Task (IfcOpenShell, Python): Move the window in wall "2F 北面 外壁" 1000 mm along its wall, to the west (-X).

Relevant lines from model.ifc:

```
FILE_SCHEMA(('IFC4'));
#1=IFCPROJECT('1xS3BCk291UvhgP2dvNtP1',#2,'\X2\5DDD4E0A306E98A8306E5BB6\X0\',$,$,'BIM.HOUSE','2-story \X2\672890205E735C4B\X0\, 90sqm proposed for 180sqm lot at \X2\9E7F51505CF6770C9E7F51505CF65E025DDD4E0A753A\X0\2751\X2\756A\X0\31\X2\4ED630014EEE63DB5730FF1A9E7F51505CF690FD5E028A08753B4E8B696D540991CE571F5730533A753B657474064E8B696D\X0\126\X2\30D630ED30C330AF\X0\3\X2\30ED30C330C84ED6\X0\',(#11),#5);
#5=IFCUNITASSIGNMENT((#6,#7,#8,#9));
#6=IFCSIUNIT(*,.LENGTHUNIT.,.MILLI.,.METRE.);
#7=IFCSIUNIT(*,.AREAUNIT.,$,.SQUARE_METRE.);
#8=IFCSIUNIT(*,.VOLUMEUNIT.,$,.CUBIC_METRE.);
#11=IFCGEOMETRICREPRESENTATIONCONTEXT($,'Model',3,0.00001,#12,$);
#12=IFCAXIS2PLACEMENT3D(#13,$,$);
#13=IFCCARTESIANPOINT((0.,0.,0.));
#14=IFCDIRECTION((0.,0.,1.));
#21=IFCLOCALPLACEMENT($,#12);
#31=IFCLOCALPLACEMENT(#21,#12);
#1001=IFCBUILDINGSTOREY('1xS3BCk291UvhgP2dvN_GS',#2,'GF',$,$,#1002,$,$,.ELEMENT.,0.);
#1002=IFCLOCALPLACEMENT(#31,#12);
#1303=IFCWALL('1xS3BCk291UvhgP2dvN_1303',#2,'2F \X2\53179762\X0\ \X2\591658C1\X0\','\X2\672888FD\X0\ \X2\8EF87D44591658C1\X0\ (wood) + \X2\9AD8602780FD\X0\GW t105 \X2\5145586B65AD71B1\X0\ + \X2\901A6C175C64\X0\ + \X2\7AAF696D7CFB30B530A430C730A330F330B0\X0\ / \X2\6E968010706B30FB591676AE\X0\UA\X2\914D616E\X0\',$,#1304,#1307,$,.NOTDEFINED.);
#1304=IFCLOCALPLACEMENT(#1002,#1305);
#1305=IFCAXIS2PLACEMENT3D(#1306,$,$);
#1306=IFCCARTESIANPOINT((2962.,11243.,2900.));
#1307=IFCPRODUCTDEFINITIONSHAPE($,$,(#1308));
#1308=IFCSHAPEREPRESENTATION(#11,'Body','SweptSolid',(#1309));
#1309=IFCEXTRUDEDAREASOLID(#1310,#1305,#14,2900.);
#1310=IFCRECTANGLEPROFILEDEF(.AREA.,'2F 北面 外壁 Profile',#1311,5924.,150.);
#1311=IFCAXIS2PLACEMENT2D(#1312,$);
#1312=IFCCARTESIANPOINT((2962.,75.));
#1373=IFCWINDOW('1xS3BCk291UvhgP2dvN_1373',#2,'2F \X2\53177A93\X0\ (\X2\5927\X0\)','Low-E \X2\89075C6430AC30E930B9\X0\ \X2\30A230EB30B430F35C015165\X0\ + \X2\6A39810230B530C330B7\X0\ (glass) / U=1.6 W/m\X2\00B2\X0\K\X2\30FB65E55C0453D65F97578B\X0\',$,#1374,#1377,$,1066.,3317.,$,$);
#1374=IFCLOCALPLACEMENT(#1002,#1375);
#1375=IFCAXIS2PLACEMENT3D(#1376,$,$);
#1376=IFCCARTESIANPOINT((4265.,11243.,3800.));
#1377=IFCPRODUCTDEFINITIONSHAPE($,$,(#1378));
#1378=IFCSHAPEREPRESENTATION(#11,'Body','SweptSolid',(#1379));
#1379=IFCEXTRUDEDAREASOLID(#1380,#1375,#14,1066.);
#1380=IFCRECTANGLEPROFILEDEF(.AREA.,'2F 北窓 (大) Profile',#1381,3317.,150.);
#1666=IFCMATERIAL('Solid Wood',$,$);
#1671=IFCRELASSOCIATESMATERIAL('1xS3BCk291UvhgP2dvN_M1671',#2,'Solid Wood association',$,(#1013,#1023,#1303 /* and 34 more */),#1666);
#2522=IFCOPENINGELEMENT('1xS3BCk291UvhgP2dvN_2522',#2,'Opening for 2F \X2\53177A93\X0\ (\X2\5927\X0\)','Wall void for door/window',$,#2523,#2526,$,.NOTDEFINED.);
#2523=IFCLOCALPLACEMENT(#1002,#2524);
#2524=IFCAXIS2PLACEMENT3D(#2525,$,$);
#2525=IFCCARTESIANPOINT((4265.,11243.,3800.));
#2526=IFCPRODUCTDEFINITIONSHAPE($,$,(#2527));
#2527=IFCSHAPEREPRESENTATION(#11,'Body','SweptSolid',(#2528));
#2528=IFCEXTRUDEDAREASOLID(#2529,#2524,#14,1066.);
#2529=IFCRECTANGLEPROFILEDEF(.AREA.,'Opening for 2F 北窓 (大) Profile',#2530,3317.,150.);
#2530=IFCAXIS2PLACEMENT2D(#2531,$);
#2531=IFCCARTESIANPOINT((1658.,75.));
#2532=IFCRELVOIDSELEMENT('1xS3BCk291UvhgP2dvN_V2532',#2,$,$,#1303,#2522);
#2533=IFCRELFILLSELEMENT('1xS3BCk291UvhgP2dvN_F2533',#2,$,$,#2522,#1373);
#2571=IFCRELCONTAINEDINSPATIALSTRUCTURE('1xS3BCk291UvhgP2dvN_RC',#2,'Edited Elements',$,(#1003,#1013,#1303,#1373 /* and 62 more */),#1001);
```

```python
import ifcopenshell
import ifcopenshell.api.geometry
import ifcopenshell.util.placement
import ifcopenshell.util.unit

model = ifcopenshell.open("model.ifc")
unit_scale = ifcopenshell.util.unit.calculate_unit_scale(model)

window = model.by_guid("1xS3BCk291UvhgP2dvN_1373")
opening = window.FillsVoids[0].RelatingOpeningElement
wall = opening.VoidsElements[0].RelatingBuildingElement

wall_matrix = ifcopenshell.util.placement.get_local_placement(wall.ObjectPlacement)
shift = wall_matrix[:3, 0] * -1 / unit_scale
before = ifcopenshell.util.placement.get_local_placement(window.ObjectPlacement)[:3, 3].copy()

# The window is not placed relative to its opening, so move both.
for product in (opening, window):
    matrix = ifcopenshell.util.placement.get_local_placement(product.ObjectPlacement)
    matrix[:3, 3] += shift
    ifcopenshell.api.geometry.edit_object_placement(model, product=product, matrix=matrix, is_si=False)

after = ifcopenshell.util.placement.get_local_placement(window.ObjectPlacement)[:3, 3]
print("window moved by", (after - before).round(3) + 0.0)

model.write("model-out.ifc")
```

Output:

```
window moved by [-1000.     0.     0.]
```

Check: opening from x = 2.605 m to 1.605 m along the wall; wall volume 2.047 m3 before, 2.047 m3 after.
